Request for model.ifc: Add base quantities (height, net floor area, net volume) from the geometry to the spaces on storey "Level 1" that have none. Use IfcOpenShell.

First a look at what the model holds.

```python
import ifcopenshell
import ifcopenshell.util.element
import ifcopenshell.util.unit

model = ifcopenshell.open("model.ifc")
print(model.schema)
for unit_type in ("LENGTHUNIT", "AREAUNIT", "VOLUMEUNIT"):
    print(unit_type, ifcopenshell.util.unit.calculate_unit_scale(model, unit_type))
storey = next(s for s in model.by_type("IfcBuildingStorey") if s.Name == "Level 1")
spaces = [e for e in ifcopenshell.util.element.get_decomposition(storey) if e.is_a("IfcSpace")]
for e in sorted(spaces, key=lambda e: e.id()):
    print(e.id(), e.is_a(), e.Name, list(ifcopenshell.util.element.get_psets(e, qtos_only=True)), sep=" | ")
```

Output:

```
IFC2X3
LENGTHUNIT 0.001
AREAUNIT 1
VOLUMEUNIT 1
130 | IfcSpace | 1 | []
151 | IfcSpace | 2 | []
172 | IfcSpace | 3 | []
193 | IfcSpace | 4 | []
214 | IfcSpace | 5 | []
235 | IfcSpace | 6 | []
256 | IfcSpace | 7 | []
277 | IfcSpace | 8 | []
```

```python
import ifcopenshell
import ifcopenshell.api.pset
import ifcopenshell.geom
import ifcopenshell.util.element
import ifcopenshell.util.shape
import ifcopenshell.util.unit

model = ifcopenshell.open("model.ifc")
unit_scale = ifcopenshell.util.unit.calculate_unit_scale(model)
area_scale = ifcopenshell.util.unit.calculate_unit_scale(model, "AREAUNIT")
volume_scale = ifcopenshell.util.unit.calculate_unit_scale(model, "VOLUMEUNIT")
settings = ifcopenshell.geom.settings()

storey = next(s for s in model.by_type("IfcBuildingStorey") if s.Name == "Level 1")
spaces = [e for e in ifcopenshell.util.element.get_decomposition(storey) if e.is_a("IfcSpace")]

for e in sorted(spaces, key=lambda e: e.id()):
    if ifcopenshell.util.element.get_psets(e, qtos_only=True, should_inherit=False):
        continue
    # Geometry comes back in metres, in the element's own axes.
    shape = ifcopenshell.geom.create_shape(settings, e)
    values = {
        "Height": ifcopenshell.util.shape.get_z(shape.geometry) / unit_scale,
        "NetFloorArea": ifcopenshell.util.shape.get_footprint_area(shape.geometry) / area_scale,
        "NetVolume": ifcopenshell.util.shape.get_volume(shape.geometry) / volume_scale,
    }
    qto = ifcopenshell.api.pset.add_qto(model, product=e, name="BaseQuantities")
    ifcopenshell.api.pset.edit_qto(model, qto=qto, properties=values)
    print(e.id(), {k: round(v, 3) for k, v in values.items()})

model.write("model_rev.ifc")
```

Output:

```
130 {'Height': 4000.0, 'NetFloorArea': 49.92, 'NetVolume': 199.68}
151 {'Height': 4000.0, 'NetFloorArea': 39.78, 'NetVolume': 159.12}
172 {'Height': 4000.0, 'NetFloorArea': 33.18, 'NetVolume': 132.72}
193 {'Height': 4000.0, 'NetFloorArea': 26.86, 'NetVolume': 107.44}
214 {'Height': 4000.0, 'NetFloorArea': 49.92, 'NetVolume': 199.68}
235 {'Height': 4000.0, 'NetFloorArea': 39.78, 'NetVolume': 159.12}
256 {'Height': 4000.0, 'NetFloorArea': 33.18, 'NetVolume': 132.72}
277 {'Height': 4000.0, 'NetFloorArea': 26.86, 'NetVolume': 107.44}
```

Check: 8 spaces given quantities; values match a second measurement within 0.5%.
